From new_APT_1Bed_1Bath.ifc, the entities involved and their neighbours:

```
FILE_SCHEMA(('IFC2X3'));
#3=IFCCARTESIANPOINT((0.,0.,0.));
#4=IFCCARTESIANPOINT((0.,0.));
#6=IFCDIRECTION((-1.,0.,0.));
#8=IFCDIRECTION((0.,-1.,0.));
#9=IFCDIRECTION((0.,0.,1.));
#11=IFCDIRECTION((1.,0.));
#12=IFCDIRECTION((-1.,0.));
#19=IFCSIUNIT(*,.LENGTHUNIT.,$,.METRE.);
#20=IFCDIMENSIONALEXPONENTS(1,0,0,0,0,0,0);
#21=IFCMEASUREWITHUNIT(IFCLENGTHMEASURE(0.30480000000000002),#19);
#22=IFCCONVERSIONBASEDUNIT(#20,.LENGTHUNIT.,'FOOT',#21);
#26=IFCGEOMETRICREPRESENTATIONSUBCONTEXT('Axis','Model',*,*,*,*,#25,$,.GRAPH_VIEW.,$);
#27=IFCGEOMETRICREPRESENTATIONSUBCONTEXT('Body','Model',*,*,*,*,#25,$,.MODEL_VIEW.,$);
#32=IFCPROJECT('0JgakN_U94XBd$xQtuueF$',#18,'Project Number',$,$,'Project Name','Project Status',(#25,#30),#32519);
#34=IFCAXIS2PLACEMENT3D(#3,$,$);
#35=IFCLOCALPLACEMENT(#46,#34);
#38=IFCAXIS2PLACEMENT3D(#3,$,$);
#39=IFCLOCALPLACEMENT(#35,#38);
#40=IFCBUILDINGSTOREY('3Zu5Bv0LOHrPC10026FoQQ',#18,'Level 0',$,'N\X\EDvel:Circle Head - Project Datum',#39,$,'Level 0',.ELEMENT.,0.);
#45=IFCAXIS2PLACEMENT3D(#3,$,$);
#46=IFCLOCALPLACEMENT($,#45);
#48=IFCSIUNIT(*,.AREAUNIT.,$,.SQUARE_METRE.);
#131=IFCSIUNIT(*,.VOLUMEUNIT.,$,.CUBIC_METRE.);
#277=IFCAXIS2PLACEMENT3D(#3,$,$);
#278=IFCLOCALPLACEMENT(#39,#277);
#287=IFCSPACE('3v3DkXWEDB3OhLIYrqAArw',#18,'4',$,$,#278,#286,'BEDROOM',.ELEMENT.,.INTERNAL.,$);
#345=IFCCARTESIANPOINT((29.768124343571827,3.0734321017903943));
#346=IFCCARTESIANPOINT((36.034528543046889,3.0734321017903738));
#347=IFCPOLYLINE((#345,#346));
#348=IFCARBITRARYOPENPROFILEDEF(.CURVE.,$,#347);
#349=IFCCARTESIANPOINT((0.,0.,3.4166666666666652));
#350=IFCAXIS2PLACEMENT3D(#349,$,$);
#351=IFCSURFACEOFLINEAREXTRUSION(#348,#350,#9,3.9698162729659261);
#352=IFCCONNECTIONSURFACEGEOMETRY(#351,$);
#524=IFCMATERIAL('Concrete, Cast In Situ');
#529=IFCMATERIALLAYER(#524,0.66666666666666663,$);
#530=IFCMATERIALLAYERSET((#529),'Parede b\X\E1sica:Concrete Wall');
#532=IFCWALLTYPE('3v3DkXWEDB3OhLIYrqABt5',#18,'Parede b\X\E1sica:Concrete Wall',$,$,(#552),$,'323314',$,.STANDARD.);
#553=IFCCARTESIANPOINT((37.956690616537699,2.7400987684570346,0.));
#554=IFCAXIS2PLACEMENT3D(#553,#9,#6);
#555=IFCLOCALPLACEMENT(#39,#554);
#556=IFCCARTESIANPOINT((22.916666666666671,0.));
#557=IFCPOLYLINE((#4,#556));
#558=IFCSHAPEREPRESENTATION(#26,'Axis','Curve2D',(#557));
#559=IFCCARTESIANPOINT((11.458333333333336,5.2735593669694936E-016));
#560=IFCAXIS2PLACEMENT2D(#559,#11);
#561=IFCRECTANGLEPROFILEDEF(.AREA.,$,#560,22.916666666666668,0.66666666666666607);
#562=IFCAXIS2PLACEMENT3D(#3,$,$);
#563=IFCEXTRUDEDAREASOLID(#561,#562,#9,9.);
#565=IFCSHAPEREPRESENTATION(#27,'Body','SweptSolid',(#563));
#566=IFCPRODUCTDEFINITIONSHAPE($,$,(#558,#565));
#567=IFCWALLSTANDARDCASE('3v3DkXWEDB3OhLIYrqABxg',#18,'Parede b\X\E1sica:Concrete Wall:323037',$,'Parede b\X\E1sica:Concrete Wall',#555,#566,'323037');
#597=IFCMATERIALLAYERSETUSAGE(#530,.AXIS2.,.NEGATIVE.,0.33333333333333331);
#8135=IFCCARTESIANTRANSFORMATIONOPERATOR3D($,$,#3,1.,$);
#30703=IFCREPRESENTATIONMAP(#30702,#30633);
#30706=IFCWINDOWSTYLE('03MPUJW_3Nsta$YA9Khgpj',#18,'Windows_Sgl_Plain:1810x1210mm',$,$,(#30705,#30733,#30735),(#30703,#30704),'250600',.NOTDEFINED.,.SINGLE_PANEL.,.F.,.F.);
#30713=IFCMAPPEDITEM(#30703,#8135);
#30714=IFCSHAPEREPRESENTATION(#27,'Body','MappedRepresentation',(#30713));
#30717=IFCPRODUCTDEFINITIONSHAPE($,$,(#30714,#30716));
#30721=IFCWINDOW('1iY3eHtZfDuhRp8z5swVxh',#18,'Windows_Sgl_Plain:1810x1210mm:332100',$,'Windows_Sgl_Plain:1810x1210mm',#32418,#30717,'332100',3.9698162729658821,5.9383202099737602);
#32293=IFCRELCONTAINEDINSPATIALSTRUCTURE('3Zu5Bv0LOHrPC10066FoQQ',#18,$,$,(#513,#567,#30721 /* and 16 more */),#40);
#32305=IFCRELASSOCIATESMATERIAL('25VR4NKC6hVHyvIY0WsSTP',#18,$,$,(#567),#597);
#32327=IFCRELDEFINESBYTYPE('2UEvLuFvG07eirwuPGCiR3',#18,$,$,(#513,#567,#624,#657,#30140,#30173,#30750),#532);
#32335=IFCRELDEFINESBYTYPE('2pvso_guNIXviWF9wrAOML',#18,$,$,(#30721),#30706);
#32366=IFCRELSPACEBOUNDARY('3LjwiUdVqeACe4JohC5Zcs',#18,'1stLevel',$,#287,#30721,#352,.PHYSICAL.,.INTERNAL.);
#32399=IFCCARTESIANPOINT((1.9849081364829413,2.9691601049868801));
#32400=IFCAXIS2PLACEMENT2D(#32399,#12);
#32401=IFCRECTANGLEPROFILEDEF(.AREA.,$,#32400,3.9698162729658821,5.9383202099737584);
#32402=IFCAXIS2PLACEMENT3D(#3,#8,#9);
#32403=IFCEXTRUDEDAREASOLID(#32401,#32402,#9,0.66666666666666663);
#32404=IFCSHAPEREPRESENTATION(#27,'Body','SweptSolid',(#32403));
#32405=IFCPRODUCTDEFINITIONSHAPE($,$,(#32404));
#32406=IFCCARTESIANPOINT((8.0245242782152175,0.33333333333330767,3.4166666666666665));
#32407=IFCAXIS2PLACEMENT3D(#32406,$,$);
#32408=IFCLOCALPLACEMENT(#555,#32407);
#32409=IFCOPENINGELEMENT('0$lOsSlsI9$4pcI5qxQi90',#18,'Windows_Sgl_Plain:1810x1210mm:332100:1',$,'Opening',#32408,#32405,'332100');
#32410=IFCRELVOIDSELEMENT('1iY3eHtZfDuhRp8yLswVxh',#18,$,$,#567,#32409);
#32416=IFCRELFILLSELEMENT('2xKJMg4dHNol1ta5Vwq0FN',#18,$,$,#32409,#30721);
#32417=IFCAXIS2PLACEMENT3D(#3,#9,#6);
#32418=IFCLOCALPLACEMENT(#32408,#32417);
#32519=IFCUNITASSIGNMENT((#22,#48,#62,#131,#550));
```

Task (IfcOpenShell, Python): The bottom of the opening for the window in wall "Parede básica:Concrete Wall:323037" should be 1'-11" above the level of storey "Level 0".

```python
import numpy as np
import ifcopenshell
import ifcopenshell.api.geometry
import ifcopenshell.geom
import ifcopenshell.util.element
import ifcopenshell.util.placement
import ifcopenshell.util.shape
import ifcopenshell.util.unit

model = ifcopenshell.open("new_APT_1Bed_1Bath.ifc")
unit_scale = ifcopenshell.util.unit.calculate_unit_scale(model)

window = model.by_guid("1iY3eHtZfDuhRp8z5swVxh")
opening = window.FillsVoids[0].RelatingOpeningElement
storey = ifcopenshell.util.element.get_container(window, ifc_class="IfcBuildingStorey")
level = ifcopenshell.util.placement.get_local_placement(storey.ObjectPlacement)[2, 3]

# The opening's origin need not be at the sill, so measure its lowest point.
shape = ifcopenshell.geom.create_shape(ifcopenshell.geom.settings(), opening)
bottom = ifcopenshell.util.shape.get_shape_bottom_elevation(shape, shape.geometry) / unit_scale
dz = level + 23 * 0.0254 / unit_scale - bottom

shift = np.array([0.0, 0.0, dz])
# The window is placed relative to its opening, so it follows when the opening moves.
matrix = ifcopenshell.util.placement.get_local_placement(opening.ObjectPlacement)
matrix[:3, 3] += shift
ifcopenshell.api.geometry.edit_object_placement(
    model, product=opening, matrix=matrix, is_si=False, should_transform_children=True
)

# Space boundary surfaces are stored in each space's coordinates; move them too.
for rel in window.ProvidesBoundaries:
    if not rel.ConnectionGeometry:
        continue
    surface = rel.ConnectionGeometry.SurfaceOnRelatingElement
    space_matrix = ifcopenshell.util.placement.get_local_placement(rel.RelatingSpace.ObjectPlacement)
    point = np.array(surface.Position.Location.Coordinates) + space_matrix[:3, :3].T @ shift
    surface.Position = model.createIfcAxis2Placement3D(
        model.createIfcCartesianPoint(point.tolist()), surface.Position.Axis, surface.Position.RefDirection
    )

print(f"moved by {dz * unit_scale:+.3f} m")

model.write("new_APT_1Bed_1Bath-out.ifc")
```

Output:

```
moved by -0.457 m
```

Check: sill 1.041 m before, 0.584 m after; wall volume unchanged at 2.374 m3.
